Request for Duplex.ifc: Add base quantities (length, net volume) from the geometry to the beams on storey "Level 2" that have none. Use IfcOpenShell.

First a look at what the model holds.

```python
import ifcopenshell
import ifcopenshell.util.element
import ifcopenshell.util.unit

model = ifcopenshell.open("Duplex.ifc")
print(model.schema)
for unit_type in ("LENGTHUNIT", "AREAUNIT", "VOLUMEUNIT"):
    print(unit_type, ifcopenshell.util.unit.calculate_unit_scale(model, unit_type))
storey = next(s for s in model.by_type("IfcBuildingStorey") if s.Name == "Level 2")
beams = [e for e in ifcopenshell.util.element.get_decomposition(storey) if e.is_a("IfcBeam")]
for e in sorted(beams, key=lambda e: e.id()):
    print(e.id(), e.is_a(), e.Name, list(ifcopenshell.util.element.get_psets(e, qtos_only=True)), sep=" | ")
```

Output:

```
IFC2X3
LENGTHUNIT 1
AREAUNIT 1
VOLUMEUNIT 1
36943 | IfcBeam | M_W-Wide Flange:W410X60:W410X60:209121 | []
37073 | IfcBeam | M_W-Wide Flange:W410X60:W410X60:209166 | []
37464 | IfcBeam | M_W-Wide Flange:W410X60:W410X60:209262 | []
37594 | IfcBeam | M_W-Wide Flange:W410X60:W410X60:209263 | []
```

```python
import ifcopenshell
import ifcopenshell.api.pset
import ifcopenshell.geom
import ifcopenshell.util.element
import ifcopenshell.util.shape
import ifcopenshell.util.unit

model = ifcopenshell.open("Duplex.ifc")
unit_scale = ifcopenshell.util.unit.calculate_unit_scale(model)
volume_scale = ifcopenshell.util.unit.calculate_unit_scale(model, "VOLUMEUNIT")
settings = ifcopenshell.geom.settings()

storey = next(s for s in model.by_type("IfcBuildingStorey") if s.Name == "Level 2")
beams = [e for e in ifcopenshell.util.element.get_decomposition(storey) if e.is_a("IfcBeam")]

for e in sorted(beams, key=lambda e: e.id()):
    if ifcopenshell.util.element.get_psets(e, qtos_only=True, should_inherit=False):
        continue
    # Geometry comes back in metres, in the element's own axes.
    shape = ifcopenshell.geom.create_shape(settings, e)
    values = {
        "Length": ifcopenshell.util.shape.get_max_xyz(shape.geometry) / unit_scale,
        "NetVolume": ifcopenshell.util.shape.get_volume(shape.geometry) / volume_scale,
    }
    qto = ifcopenshell.api.pset.add_qto(model, product=e, name="BaseQuantities")
    ifcopenshell.api.pset.edit_qto(model, qto=qto, properties=values)
    print(e.id(), {k: round(v, 3) for k, v in values.items()})

model.write("Duplex_rev.ifc")
```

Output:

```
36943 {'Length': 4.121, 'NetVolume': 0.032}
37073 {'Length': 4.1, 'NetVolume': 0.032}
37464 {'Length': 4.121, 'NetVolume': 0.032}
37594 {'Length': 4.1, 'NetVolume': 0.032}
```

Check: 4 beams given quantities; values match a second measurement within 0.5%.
